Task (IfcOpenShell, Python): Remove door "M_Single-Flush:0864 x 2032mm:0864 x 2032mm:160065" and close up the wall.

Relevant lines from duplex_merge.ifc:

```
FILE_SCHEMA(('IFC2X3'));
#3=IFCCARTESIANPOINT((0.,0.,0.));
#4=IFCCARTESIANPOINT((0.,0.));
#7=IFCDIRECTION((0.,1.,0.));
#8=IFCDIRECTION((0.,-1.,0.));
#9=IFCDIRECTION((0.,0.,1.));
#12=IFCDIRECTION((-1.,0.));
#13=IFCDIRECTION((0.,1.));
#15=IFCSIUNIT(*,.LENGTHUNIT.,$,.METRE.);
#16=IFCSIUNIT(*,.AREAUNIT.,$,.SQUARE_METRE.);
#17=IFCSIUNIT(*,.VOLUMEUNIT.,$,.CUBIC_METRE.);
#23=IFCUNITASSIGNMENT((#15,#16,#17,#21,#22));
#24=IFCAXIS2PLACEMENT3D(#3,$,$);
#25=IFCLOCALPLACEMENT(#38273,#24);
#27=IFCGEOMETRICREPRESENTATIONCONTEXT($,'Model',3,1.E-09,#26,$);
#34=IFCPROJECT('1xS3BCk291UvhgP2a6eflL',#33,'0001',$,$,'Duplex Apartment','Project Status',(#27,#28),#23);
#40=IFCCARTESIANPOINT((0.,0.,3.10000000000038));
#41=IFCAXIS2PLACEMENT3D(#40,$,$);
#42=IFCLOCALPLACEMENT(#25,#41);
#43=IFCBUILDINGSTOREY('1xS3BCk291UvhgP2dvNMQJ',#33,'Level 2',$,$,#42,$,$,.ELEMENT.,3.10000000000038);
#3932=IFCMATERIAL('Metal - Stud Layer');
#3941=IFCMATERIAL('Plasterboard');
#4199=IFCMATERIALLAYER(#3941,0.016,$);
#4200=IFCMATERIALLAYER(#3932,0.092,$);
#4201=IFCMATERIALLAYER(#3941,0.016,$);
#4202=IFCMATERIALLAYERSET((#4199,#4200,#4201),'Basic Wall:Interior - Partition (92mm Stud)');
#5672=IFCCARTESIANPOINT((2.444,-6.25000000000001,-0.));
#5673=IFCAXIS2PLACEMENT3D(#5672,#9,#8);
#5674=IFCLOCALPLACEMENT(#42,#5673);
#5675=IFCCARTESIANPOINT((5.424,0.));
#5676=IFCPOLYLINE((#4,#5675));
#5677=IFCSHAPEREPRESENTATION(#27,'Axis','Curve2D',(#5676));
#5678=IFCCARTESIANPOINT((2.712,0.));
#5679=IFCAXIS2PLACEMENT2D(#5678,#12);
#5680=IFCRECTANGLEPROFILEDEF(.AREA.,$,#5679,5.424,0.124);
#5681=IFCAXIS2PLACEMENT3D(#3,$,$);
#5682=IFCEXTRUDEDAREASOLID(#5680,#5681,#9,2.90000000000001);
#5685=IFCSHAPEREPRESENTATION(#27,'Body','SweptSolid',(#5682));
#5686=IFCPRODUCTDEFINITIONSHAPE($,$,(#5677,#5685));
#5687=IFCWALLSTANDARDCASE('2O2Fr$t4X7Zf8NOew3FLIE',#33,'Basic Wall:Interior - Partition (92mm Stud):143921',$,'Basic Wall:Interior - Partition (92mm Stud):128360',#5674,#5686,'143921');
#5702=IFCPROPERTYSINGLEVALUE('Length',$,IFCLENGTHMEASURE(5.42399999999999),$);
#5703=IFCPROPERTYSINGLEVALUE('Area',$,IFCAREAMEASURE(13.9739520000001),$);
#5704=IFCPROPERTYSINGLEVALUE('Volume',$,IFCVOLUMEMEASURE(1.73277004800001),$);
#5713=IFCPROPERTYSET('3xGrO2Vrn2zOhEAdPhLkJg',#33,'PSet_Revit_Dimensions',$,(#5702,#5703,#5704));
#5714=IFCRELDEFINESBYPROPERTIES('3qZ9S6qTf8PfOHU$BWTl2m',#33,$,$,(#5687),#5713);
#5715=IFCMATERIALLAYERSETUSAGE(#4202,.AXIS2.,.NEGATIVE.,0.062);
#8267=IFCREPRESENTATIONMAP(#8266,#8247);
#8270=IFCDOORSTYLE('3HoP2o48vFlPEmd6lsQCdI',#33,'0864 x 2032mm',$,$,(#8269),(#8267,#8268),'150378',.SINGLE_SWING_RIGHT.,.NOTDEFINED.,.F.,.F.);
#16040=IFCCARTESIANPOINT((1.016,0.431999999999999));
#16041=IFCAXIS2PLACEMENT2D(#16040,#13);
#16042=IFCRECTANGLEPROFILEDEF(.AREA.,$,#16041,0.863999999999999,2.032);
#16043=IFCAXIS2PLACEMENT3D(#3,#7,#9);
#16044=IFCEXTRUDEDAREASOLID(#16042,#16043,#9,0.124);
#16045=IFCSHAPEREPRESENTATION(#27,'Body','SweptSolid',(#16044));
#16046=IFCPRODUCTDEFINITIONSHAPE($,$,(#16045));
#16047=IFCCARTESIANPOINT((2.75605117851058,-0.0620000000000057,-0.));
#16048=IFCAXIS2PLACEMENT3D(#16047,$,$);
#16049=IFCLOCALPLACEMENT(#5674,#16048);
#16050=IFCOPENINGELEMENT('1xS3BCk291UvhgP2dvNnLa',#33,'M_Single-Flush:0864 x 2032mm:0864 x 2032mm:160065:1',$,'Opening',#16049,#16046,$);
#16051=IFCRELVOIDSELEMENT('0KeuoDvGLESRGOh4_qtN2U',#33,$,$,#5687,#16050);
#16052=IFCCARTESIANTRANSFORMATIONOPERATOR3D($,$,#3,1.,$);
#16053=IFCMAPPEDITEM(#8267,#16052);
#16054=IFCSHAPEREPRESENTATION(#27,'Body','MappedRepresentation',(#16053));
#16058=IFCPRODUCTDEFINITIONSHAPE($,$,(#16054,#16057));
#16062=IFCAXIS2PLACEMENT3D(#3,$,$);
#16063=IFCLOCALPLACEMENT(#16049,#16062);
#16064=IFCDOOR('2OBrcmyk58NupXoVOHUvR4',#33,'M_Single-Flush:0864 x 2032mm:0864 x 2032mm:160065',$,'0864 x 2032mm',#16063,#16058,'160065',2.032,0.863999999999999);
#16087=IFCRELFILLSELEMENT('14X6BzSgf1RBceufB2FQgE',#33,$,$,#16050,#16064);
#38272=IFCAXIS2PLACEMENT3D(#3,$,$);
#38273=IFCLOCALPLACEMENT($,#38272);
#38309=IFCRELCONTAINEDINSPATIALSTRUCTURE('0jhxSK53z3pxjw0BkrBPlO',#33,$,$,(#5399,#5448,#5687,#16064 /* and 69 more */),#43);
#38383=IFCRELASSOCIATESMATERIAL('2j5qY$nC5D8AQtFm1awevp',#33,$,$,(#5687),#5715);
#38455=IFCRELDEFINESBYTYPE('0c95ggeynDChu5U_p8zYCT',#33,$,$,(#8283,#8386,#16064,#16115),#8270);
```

```python
import ifcopenshell
import ifcopenshell.api.feature
import ifcopenshell.api.pset
import ifcopenshell.api.root
import ifcopenshell.geom
import ifcopenshell.util.element
import ifcopenshell.util.shape
import ifcopenshell.util.unit

model = ifcopenshell.open("duplex_merge.ifc")
area_scale = ifcopenshell.util.unit.calculate_unit_scale(model, "AREAUNIT")
volume_scale = ifcopenshell.util.unit.calculate_unit_scale(model, "VOLUMEUNIT")
settings = ifcopenshell.geom.settings()


def volume(element):
    """Net volume in cubic metres, openings subtracted."""
    shape = ifcopenshell.geom.create_shape(settings, element)
    return ifcopenshell.util.shape.get_volume(shape.geometry)


door = model.by_guid("2OBrcmyk58NupXoVOHUvR4")
opening = door.FillsVoids[0].RelatingOpeningElement
wall = opening.VoidsElements[0].RelatingBuildingElement
before = volume(wall)

ifcopenshell.api.root.remove_product(model, product=door)
ifcopenshell.api.feature.remove_feature(model, feature=opening)

after = volume(wall)
thickness = 0.124  # wall thickness in metres

# Update the wall's stored quantities.
pset = model.by_id(ifcopenshell.util.element.get_pset(wall, "PSet_Revit_Dimensions", should_inherit=False)["id"])
ifcopenshell.api.pset.edit_pset(model, pset=pset, properties={
    "Area": model.create_entity("IfcAreaMeasure", after / thickness / area_scale),
    "Volume": model.create_entity("IfcVolumeMeasure", after / volume_scale),
})

print(f"wall volume {before:.3f} -> {after:.3f} m3")

model.write("duplex_merge_v2.ifc")
```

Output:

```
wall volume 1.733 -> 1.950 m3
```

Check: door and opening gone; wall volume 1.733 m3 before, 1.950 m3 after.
